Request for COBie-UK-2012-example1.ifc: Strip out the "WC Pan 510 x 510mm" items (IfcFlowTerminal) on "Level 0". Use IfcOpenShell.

First a look at what the model holds.

```python
import ifcopenshell
import ifcopenshell.util.element

model = ifcopenshell.open("COBie-UK-2012-example1.ifc")
print(model.schema)
storey = next(s for s in model.by_type("IfcBuildingStorey") if s.Name == "Level 0")
terminals = [e for e in ifcopenshell.util.element.get_decomposition(storey) if e.is_a("IfcFlowTerminal")]
seen = {}
for e in terminals:
    element_type = ifcopenshell.util.element.get_type(e)
    name = element_type.Name if element_type not in (None, e) else None
    seen[name] = seen.get(name, 0) + 1
for name, count in sorted(seen.items(), key=str):
    print(count, "x", name)
```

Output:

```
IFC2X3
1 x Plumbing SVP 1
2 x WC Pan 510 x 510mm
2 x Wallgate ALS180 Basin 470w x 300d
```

```python
import ifcopenshell
import ifcopenshell.api.root
import ifcopenshell.util.element

model = ifcopenshell.open("COBie-UK-2012-example1.ifc")

storey = next(s for s in model.by_type("IfcBuildingStorey") if s.Name == "Level 0")
terminals = [e for e in ifcopenshell.util.element.get_decomposition(storey) if e.is_a("IfcFlowTerminal")]
targets = [e for e in terminals if (t := ifcopenshell.util.element.get_type(e)) not in (None, e) and t.Name == "WC Pan 510 x 510mm"]

for e in targets:
    ifcopenshell.api.root.remove_product(model, product=e)
print(len(targets), "removed")

model.write("COBie-UK-2012-example1_updated.ifc")
```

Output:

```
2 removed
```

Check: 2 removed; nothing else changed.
